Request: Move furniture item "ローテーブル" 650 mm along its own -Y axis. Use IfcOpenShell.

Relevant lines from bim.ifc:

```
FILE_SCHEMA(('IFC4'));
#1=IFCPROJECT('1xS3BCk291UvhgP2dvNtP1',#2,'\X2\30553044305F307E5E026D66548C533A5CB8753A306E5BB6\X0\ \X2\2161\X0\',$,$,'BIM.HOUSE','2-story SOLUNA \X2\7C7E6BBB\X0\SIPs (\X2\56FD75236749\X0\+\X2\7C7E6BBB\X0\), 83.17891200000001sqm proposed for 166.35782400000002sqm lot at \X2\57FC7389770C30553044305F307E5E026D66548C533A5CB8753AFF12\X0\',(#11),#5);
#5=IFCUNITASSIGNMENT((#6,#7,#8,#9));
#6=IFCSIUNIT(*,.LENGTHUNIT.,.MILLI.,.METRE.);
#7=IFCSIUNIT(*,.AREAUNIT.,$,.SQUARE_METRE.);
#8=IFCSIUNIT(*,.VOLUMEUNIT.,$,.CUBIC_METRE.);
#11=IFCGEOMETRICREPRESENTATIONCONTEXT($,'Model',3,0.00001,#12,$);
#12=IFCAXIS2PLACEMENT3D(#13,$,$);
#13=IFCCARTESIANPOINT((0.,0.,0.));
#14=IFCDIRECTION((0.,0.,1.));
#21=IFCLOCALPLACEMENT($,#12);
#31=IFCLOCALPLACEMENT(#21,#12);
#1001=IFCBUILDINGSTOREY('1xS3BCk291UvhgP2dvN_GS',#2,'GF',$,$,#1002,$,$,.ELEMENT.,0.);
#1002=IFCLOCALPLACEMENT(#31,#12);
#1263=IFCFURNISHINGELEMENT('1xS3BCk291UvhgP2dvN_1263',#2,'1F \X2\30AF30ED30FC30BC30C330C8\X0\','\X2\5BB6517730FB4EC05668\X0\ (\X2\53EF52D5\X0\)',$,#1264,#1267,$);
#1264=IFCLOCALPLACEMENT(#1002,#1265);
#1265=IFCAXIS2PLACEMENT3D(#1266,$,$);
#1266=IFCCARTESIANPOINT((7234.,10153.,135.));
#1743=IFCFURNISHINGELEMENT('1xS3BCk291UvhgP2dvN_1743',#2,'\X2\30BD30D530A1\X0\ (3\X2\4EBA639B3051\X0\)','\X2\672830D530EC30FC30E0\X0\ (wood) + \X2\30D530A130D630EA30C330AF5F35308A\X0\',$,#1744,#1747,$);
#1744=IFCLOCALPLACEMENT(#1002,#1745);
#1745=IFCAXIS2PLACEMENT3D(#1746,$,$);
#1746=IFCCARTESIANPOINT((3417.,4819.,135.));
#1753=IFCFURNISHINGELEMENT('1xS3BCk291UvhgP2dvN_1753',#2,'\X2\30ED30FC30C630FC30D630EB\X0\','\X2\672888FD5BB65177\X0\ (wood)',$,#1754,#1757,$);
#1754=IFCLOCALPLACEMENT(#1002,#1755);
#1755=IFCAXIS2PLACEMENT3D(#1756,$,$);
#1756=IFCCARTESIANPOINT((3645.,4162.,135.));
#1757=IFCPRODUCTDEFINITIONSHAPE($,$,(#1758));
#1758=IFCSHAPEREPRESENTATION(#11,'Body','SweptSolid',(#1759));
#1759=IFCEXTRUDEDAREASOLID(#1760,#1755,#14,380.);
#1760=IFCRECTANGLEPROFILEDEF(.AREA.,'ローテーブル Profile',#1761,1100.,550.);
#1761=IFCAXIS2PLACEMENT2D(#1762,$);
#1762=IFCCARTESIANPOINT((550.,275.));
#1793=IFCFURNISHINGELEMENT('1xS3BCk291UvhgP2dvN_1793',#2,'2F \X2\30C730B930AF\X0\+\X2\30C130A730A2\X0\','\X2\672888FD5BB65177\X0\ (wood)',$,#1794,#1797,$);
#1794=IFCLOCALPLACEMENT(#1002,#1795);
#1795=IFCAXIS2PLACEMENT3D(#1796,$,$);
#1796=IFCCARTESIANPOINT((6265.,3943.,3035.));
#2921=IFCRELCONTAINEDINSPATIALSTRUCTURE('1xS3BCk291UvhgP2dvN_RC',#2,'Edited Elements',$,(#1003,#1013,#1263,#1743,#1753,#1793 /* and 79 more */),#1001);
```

```python
import ifcopenshell
import ifcopenshell.api.geometry
import ifcopenshell.util.placement
import ifcopenshell.util.unit

model = ifcopenshell.open("bim.ifc")
unit_scale = ifcopenshell.util.unit.calculate_unit_scale(model)

item = model.by_id(1753)
matrix = ifcopenshell.util.placement.get_local_placement(item.ObjectPlacement)
matrix[:3, 3] -= matrix[:3, 1] * 0.65 / unit_scale
ifcopenshell.api.geometry.edit_object_placement(model, product=item, matrix=matrix, is_si=False)

print(ifcopenshell.util.placement.get_local_placement(item.ObjectPlacement).round(3) + 0.0)

model.write("bim_updated.ifc")
```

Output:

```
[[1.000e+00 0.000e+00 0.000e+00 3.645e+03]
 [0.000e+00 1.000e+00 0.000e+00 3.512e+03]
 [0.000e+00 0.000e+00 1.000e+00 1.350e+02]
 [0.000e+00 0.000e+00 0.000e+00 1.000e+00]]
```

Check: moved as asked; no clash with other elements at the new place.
